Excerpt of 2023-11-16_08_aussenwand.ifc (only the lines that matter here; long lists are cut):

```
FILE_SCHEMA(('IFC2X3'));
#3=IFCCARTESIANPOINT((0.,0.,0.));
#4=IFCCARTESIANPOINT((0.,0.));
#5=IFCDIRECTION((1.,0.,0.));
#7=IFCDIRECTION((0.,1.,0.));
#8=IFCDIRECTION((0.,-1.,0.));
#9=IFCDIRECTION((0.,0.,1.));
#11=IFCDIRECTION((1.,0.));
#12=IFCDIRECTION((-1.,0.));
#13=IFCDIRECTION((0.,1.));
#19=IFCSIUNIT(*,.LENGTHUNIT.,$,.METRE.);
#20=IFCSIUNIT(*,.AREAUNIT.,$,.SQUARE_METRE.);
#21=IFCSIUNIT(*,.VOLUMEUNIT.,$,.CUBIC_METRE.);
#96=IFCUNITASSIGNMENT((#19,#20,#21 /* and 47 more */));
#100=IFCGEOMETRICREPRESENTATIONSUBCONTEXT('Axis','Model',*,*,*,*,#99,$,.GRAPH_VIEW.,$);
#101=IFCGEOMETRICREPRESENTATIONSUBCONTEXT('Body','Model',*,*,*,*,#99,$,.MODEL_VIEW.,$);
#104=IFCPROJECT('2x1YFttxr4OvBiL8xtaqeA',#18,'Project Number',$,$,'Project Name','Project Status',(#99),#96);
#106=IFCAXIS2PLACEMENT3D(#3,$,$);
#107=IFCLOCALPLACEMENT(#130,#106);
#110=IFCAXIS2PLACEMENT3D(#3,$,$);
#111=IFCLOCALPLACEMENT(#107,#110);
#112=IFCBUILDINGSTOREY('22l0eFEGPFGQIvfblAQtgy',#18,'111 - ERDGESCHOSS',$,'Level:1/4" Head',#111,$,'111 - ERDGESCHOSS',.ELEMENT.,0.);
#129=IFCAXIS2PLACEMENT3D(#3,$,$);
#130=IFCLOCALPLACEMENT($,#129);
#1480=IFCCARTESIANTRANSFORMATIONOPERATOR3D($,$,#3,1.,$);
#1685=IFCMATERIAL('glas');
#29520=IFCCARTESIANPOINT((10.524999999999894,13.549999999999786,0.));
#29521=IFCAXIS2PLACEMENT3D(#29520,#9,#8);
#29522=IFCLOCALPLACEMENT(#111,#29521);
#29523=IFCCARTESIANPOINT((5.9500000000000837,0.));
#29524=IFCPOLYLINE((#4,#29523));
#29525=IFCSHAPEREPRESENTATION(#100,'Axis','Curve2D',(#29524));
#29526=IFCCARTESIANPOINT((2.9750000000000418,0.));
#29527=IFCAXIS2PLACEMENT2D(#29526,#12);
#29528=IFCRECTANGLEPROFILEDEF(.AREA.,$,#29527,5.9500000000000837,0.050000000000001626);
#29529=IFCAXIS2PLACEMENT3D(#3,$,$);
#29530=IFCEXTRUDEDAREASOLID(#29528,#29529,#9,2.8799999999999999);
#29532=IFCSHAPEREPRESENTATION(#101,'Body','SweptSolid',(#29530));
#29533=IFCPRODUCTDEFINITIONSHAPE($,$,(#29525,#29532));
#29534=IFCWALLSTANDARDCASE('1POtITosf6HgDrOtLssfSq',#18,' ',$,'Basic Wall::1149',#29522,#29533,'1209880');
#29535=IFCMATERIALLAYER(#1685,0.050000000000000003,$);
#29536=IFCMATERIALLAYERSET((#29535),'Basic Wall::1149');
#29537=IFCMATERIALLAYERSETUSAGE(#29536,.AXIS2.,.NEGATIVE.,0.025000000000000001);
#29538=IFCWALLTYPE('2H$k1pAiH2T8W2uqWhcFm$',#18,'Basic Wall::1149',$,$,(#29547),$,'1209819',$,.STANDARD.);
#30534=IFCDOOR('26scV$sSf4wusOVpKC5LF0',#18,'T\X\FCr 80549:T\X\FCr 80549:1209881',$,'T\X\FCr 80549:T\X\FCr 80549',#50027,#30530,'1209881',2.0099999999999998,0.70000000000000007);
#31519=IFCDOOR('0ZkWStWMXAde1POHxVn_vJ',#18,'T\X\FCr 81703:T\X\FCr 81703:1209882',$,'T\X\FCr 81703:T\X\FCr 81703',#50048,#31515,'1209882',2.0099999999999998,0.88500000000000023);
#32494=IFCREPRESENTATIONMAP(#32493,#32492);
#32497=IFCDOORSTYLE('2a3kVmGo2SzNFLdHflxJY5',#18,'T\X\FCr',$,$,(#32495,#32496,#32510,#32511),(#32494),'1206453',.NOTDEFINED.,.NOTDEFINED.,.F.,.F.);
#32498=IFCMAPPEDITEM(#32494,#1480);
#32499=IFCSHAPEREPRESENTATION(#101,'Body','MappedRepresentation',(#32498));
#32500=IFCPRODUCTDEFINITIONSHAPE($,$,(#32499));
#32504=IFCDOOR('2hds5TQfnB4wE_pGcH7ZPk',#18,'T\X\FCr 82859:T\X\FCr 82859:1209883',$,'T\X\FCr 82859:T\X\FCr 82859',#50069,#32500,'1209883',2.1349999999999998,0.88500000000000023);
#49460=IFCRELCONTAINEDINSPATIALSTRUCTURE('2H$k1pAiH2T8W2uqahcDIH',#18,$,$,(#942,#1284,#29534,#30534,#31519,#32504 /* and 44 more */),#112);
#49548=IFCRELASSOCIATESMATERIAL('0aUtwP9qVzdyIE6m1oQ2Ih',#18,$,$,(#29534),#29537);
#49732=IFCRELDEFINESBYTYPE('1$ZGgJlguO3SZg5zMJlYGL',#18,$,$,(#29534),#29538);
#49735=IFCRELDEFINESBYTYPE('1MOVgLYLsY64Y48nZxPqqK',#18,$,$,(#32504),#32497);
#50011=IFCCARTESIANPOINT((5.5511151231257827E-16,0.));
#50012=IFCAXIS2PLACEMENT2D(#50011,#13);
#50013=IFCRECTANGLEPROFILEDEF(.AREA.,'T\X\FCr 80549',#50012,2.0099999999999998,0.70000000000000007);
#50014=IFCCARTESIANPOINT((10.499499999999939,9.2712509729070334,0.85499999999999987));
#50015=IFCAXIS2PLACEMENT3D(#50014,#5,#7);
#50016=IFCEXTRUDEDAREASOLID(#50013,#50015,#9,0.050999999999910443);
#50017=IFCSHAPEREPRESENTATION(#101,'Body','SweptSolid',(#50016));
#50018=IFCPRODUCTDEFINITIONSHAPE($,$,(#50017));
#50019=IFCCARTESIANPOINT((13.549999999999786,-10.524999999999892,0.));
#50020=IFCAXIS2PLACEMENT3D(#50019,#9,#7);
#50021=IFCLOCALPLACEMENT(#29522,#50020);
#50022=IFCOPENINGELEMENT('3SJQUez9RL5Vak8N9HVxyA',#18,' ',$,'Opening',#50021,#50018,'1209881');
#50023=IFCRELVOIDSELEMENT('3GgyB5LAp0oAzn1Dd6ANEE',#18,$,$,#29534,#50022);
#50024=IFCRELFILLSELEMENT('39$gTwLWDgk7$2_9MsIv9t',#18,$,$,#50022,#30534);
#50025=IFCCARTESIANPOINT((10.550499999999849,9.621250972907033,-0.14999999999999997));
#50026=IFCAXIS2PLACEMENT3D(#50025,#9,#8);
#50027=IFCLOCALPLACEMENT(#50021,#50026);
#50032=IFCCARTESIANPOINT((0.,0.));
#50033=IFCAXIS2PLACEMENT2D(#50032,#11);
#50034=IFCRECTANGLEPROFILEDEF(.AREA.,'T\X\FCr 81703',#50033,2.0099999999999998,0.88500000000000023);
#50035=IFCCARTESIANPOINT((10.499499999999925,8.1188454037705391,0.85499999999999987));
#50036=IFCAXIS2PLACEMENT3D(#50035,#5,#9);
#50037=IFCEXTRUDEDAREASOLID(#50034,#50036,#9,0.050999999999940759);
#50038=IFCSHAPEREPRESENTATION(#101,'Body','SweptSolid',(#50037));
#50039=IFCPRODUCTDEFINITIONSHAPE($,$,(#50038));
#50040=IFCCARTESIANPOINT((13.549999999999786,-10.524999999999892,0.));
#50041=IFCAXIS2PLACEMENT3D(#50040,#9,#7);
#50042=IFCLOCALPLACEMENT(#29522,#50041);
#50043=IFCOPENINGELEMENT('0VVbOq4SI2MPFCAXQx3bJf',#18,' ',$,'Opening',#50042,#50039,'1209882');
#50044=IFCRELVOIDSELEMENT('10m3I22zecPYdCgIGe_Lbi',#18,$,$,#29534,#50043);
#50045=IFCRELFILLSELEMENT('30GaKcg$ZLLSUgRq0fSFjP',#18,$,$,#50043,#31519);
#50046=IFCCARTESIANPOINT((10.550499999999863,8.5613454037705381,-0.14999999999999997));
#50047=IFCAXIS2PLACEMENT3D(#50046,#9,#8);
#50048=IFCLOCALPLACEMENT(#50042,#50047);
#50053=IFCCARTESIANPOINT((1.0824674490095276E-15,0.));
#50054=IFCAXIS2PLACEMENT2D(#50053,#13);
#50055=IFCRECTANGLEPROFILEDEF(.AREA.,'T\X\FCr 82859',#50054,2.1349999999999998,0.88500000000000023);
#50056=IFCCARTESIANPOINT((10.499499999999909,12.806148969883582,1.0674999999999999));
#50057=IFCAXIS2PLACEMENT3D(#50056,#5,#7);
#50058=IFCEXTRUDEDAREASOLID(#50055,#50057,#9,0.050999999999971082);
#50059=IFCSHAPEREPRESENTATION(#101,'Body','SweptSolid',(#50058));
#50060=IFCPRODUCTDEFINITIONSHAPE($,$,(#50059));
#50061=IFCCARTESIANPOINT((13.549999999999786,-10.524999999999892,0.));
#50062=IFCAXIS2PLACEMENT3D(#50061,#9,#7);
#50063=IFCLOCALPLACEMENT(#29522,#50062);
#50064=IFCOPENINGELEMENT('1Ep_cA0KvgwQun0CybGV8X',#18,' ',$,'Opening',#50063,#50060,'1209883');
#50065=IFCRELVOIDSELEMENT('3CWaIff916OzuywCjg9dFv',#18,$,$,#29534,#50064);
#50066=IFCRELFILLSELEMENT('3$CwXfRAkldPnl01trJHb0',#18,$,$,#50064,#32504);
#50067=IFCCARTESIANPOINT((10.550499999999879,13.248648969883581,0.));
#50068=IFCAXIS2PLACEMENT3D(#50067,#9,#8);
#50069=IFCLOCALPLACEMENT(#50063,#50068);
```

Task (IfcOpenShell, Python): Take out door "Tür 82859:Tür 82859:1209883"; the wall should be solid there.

```python
import ifcopenshell
import ifcopenshell.api.feature
import ifcopenshell.api.root
import ifcopenshell.geom
import ifcopenshell.util.shape

model = ifcopenshell.open("2023-11-16_08_aussenwand.ifc")
settings = ifcopenshell.geom.settings()


def volume(element):
    """Net volume in cubic metres, openings subtracted."""
    shape = ifcopenshell.geom.create_shape(settings, element)
    return ifcopenshell.util.shape.get_volume(shape.geometry)


door = model.by_id(32504)
opening = door.FillsVoids[0].RelatingOpeningElement
wall = opening.VoidsElements[0].RelatingBuildingElement
before = volume(wall)

ifcopenshell.api.root.remove_product(model, product=door)
ifcopenshell.api.feature.remove_feature(model, feature=opening)

after = volume(wall)

print(f"wall volume {before:.3f} -> {after:.3f} m3")

model.write("2023-11-16_08_aussenwand_rev.ifc")
```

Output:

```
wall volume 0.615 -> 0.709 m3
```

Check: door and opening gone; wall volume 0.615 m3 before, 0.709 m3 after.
